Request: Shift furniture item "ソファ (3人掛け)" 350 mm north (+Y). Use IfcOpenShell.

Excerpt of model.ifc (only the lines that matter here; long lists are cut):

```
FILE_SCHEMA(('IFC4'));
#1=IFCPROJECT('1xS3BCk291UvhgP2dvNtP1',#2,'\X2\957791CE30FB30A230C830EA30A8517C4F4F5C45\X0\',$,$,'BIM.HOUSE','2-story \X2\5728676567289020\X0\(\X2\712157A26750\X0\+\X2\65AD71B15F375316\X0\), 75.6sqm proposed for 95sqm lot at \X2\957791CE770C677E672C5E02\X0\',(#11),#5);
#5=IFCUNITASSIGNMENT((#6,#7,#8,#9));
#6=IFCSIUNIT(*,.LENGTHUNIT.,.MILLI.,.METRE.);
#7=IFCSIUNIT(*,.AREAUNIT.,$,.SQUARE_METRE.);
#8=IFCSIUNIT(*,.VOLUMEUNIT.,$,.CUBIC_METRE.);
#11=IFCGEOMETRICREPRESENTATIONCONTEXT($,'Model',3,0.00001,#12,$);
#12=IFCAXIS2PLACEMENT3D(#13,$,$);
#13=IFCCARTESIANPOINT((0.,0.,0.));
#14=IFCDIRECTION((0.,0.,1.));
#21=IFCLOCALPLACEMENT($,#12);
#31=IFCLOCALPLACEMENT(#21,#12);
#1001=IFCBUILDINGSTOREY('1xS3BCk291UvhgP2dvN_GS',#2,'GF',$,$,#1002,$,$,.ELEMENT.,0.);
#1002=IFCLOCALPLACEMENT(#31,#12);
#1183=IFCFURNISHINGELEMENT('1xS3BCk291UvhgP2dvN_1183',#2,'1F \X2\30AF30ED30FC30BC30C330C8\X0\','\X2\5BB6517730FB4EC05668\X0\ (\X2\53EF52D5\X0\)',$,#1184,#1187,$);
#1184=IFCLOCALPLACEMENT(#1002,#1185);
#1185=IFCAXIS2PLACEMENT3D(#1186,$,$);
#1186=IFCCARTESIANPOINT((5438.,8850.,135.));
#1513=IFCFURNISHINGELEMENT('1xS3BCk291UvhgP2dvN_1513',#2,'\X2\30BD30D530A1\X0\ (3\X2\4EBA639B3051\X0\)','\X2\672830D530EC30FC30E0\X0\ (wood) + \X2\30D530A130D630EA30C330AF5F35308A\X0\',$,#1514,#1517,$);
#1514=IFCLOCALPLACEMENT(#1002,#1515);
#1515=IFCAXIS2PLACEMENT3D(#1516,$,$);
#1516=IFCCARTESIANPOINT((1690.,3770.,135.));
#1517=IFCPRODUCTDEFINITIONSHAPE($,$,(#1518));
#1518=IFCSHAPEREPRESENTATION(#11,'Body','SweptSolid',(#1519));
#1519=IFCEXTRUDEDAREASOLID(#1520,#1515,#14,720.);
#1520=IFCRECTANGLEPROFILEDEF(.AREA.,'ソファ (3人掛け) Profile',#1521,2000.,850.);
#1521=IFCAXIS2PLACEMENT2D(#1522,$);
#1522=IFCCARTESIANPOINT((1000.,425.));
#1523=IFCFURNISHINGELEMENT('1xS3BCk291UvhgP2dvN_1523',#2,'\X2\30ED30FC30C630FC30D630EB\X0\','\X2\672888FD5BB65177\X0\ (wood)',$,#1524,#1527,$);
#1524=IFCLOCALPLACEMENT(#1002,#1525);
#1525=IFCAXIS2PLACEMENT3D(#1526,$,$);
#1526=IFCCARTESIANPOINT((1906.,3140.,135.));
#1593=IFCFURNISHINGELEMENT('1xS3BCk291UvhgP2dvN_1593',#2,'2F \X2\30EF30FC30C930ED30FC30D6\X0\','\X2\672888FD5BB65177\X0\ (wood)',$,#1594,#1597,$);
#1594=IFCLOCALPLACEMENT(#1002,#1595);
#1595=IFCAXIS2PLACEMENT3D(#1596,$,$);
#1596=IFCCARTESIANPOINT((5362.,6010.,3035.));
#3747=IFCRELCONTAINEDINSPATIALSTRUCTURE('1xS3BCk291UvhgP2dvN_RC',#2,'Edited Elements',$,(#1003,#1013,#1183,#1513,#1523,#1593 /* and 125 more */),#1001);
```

```python
import ifcopenshell
import ifcopenshell.api.geometry
import ifcopenshell.util.placement
import ifcopenshell.util.unit

model = ifcopenshell.open("model.ifc")
unit_scale = ifcopenshell.util.unit.calculate_unit_scale(model)

item = model.by_id(1513)
matrix = ifcopenshell.util.placement.get_local_placement(item.ObjectPlacement)
matrix[1, 3] += 0.35 / unit_scale
ifcopenshell.api.geometry.edit_object_placement(model, product=item, matrix=matrix, is_si=False)

print(ifcopenshell.util.placement.get_local_placement(item.ObjectPlacement).round(3) + 0.0)

model.write("model-out.ifc")
```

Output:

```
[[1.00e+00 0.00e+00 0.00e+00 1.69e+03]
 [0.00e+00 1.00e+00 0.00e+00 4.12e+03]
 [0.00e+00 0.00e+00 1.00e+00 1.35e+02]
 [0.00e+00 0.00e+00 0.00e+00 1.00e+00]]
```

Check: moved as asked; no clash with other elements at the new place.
